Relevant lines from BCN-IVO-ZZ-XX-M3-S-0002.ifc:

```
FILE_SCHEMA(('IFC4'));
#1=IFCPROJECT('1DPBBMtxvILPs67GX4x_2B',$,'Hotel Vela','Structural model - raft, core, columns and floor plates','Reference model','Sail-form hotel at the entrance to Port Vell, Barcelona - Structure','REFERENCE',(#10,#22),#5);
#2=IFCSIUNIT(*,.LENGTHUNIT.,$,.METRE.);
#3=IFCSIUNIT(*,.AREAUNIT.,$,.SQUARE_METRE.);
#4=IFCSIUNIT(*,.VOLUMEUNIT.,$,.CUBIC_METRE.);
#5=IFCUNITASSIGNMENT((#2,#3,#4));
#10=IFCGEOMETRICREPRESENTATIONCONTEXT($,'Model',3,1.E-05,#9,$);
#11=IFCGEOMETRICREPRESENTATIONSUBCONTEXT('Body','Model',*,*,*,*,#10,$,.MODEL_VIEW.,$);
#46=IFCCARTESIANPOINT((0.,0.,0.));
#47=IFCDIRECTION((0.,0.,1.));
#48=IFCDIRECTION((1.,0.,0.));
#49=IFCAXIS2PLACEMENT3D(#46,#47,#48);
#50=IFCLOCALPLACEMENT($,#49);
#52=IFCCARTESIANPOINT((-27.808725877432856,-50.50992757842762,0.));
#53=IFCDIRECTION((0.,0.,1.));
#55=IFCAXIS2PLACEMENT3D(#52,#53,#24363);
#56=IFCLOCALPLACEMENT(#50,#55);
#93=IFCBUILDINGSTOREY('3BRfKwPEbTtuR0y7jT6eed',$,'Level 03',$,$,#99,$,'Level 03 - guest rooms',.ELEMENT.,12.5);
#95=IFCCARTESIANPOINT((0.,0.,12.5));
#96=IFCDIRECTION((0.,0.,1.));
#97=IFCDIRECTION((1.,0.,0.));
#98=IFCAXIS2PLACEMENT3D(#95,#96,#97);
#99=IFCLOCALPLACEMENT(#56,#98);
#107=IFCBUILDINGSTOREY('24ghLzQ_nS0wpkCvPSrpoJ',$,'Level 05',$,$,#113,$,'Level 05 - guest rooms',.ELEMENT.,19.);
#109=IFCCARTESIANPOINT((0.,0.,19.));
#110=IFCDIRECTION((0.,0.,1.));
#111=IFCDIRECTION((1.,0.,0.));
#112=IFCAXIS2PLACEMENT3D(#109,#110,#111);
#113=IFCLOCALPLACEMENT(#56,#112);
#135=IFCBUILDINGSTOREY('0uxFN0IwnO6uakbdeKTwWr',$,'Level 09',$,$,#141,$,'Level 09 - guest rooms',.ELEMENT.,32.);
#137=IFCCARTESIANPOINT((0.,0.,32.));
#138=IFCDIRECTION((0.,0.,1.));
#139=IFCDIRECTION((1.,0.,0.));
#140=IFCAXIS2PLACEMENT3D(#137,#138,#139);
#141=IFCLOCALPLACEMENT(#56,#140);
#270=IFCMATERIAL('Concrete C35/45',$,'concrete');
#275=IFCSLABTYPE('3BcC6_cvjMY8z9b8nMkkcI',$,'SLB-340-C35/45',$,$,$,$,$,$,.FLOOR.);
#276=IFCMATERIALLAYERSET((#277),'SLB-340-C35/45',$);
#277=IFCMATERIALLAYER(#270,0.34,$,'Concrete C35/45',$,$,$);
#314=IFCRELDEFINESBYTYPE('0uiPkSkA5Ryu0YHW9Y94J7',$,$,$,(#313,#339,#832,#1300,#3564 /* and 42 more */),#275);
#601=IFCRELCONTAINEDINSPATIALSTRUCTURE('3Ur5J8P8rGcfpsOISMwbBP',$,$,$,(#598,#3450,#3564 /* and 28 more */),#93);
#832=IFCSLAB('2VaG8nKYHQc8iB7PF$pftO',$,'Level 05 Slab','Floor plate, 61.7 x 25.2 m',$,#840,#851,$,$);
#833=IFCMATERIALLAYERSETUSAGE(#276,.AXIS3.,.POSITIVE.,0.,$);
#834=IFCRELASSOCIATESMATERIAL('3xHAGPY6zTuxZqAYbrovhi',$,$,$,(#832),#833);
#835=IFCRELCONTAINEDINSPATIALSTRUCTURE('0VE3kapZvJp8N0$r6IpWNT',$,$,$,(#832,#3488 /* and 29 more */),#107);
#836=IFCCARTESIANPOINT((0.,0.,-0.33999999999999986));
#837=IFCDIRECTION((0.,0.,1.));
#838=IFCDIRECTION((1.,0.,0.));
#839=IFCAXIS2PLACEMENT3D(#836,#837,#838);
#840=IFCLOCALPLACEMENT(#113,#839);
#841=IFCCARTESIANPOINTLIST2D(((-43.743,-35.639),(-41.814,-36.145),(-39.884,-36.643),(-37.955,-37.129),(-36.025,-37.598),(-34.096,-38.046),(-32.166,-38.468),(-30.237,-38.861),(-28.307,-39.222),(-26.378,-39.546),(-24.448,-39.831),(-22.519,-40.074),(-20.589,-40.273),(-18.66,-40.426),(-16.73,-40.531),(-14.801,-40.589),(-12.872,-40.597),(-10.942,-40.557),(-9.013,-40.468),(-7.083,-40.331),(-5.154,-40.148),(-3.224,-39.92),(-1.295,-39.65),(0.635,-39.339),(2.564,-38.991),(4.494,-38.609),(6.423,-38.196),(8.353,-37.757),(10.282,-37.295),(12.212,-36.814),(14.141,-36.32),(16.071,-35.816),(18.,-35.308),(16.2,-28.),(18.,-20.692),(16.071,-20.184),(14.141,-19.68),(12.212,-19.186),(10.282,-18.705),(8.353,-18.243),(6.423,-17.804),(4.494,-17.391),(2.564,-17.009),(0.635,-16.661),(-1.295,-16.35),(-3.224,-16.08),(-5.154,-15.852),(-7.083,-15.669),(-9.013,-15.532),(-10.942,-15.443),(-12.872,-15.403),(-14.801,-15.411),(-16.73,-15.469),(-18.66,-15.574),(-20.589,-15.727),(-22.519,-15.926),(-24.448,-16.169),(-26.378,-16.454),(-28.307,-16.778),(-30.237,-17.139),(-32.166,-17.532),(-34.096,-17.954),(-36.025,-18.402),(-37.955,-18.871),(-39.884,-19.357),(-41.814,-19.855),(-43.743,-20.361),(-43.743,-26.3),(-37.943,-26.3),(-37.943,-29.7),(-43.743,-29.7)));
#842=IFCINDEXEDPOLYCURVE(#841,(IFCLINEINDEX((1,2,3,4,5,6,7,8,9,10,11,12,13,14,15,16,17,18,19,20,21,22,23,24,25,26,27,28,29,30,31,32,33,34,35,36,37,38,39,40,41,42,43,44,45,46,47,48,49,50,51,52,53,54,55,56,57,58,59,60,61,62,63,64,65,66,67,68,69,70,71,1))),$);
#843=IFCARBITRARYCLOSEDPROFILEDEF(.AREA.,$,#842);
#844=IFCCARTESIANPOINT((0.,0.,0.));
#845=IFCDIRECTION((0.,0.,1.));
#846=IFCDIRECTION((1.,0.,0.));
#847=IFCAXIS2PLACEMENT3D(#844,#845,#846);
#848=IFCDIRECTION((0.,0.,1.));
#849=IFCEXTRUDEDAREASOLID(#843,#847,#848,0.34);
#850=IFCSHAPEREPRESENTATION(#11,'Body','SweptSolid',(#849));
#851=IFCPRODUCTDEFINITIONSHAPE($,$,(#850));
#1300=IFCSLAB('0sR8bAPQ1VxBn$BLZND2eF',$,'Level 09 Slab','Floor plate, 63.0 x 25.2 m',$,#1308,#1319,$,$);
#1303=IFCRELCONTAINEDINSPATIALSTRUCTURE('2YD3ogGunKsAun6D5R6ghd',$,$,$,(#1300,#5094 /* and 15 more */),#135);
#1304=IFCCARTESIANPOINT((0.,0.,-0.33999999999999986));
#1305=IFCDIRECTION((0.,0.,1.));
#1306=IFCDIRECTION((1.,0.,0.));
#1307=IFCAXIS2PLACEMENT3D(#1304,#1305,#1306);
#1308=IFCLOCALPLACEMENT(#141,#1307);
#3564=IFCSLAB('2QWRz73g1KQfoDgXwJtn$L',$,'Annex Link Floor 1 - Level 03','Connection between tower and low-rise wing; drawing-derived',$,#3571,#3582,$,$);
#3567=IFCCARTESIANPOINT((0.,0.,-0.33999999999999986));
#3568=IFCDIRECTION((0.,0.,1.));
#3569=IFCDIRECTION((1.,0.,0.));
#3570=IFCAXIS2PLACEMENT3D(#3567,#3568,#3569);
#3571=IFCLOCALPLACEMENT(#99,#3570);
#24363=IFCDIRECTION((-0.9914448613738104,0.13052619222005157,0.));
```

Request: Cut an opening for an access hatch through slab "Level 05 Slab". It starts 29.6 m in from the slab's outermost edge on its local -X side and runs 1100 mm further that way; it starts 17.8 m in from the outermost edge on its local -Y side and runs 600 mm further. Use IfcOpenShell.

```python
import numpy as np
import ifcopenshell
import ifcopenshell.api.feature
import ifcopenshell.api.geometry
import ifcopenshell.api.root
import ifcopenshell.geom
import ifcopenshell.util.placement
import ifcopenshell.util.representation
import ifcopenshell.util.shape
import ifcopenshell.util.unit

model = ifcopenshell.open("BCN-IVO-ZZ-XX-M3-S-0002.ifc")
unit_scale = ifcopenshell.util.unit.calculate_unit_scale(model)
settings = ifcopenshell.geom.settings()


def volume(element):
    """Net volume in cubic metres, openings subtracted."""
    shape = ifcopenshell.geom.create_shape(settings, element)
    return ifcopenshell.util.shape.get_volume(shape.geometry)


slab = model.by_id(832)
before = volume(slab)

# Extent in the slab's own axes, in metres. The edges named are its -X and -Y sides.
slab_shape = ifcopenshell.geom.create_shape(settings, slab)
vertices = ifcopenshell.util.shape.get_vertices(slab_shape.geometry)
x_min, y_min, bottom = vertices.min(axis=0)
top = vertices[:, 2].max()

opening = ifcopenshell.api.root.create_entity(model, ifc_class="IfcOpeningElement", name="Access hatch opening", predefined_type="OPENING")
context = ifcopenshell.util.representation.get_context(model, "Model", "Body", "MODEL_VIEW")
width, depth = 1.1, 0.6
outline = [(0.0, 0.0), (width, 0.0), (width, depth), (0.0, depth), (0.0, 0.0)]
# Overshoot both faces by 50 mm so the cut is clean.
shape = ifcopenshell.api.geometry.add_slab_representation(
    model, context=context, depth=top - bottom + 0.1, polyline=outline
)
ifcopenshell.api.geometry.assign_representation(model, product=opening, representation=shape)

matrix = ifcopenshell.util.placement.get_local_placement(slab.ObjectPlacement)
matrix[:, 3] = matrix @ np.append(np.array([x_min + 29.6, y_min + 17.8, bottom - 0.05]) / unit_scale, 1.0)
ifcopenshell.api.geometry.edit_object_placement(model, product=opening, matrix=matrix, is_si=False)
ifcopenshell.api.feature.add_feature(model, feature=opening, element=slab)

after = volume(slab)

print(f"slab volume {before:.3f} -> {after:.3f} m3")

model.write("BCN-IVO-ZZ-XX-M3-S-0002_v2.ifc")
```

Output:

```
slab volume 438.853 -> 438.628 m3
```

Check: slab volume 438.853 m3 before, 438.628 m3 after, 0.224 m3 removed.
